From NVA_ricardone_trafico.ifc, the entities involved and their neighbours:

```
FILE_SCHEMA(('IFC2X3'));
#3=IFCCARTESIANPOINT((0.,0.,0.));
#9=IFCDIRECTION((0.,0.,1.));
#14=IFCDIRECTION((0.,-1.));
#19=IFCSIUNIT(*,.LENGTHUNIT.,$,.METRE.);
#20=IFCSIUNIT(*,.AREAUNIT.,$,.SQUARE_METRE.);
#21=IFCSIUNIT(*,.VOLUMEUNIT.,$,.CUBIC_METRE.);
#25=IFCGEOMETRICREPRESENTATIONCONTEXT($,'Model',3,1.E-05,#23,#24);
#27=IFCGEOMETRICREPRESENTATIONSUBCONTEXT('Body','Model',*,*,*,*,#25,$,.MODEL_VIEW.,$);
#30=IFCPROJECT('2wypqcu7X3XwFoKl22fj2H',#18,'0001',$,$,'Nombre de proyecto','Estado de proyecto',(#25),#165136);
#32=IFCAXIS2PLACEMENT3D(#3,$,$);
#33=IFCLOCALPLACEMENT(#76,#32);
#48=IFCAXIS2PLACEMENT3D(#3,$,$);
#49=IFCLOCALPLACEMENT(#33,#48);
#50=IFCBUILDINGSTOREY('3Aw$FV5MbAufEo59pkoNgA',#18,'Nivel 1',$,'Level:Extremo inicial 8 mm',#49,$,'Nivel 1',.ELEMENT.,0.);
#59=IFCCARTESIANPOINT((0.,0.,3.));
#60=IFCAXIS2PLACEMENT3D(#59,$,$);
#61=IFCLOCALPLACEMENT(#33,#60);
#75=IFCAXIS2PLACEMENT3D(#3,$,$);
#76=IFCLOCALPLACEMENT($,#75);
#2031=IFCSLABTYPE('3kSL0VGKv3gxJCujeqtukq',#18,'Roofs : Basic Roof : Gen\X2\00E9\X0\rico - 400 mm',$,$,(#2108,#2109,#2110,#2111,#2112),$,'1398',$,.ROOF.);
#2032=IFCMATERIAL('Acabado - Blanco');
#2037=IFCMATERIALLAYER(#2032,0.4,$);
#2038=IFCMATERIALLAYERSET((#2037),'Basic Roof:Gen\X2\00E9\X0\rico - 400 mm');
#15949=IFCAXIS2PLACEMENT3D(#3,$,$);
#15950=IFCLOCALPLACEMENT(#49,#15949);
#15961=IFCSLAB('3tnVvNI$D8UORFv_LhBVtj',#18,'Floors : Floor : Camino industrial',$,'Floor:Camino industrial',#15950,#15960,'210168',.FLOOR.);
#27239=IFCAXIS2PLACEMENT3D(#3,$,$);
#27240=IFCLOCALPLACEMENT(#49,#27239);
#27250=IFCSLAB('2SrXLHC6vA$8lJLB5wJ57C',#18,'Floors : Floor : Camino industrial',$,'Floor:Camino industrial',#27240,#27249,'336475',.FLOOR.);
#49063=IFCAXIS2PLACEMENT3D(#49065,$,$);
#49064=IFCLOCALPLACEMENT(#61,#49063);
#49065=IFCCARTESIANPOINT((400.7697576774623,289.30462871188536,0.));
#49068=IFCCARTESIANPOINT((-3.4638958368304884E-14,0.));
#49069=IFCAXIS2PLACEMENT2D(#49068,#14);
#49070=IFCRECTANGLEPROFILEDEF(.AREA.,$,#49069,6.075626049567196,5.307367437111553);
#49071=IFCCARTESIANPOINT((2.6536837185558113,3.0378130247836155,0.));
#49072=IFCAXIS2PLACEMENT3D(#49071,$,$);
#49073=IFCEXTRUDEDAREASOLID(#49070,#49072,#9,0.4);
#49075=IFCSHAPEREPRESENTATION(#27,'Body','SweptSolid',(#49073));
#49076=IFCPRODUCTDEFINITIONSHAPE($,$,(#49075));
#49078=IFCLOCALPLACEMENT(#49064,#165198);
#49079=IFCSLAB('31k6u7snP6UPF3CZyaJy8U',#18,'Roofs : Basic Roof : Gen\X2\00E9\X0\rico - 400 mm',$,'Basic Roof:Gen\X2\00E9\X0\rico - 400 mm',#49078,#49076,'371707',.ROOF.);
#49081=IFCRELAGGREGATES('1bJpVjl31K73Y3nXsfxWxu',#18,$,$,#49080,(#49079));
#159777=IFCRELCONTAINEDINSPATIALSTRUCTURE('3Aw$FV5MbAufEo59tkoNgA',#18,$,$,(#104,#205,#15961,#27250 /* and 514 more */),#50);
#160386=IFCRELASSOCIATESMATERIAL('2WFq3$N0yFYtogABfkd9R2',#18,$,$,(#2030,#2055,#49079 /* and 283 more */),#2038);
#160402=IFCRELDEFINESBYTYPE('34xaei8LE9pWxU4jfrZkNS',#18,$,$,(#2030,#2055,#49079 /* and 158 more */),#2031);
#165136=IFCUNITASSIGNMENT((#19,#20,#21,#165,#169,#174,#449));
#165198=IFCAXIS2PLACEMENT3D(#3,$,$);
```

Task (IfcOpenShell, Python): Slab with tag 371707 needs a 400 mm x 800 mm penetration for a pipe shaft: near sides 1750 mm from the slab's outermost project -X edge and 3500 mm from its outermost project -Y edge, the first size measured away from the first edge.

```python
import numpy as np
import ifcopenshell
import ifcopenshell.api.feature
import ifcopenshell.api.geometry
import ifcopenshell.api.root
import ifcopenshell.geom
import ifcopenshell.util.placement
import ifcopenshell.util.representation
import ifcopenshell.util.shape
import ifcopenshell.util.unit

model = ifcopenshell.open("NVA_ricardone_trafico.ifc")
unit_scale = ifcopenshell.util.unit.calculate_unit_scale(model)
settings = ifcopenshell.geom.settings()


def volume(element):
    """Net volume in cubic metres, openings subtracted."""
    shape = ifcopenshell.geom.create_shape(settings, element)
    return ifcopenshell.util.shape.get_volume(shape.geometry)


slab = model.by_id(49079)
before = volume(slab)

# Extent in the slab's own axes, in metres. The edges named are its -X and -Y sides.
slab_shape = ifcopenshell.geom.create_shape(settings, slab)
vertices = ifcopenshell.util.shape.get_vertices(slab_shape.geometry)
x_min, y_min, bottom = vertices.min(axis=0)
top = vertices[:, 2].max()

opening = ifcopenshell.api.root.create_entity(model, ifc_class="IfcOpeningElement", name="Pipe shaft opening")
context = ifcopenshell.util.representation.get_context(model, "Model", "Body", "MODEL_VIEW")
width, depth = 0.4, 0.8
outline = [(0.0, 0.0), (width, 0.0), (width, depth), (0.0, depth), (0.0, 0.0)]
# Overshoot both faces by 50 mm so the cut is clean.
shape = ifcopenshell.api.geometry.add_slab_representation(
    model, context=context, depth=top - bottom + 0.1, polyline=outline
)
ifcopenshell.api.geometry.assign_representation(model, product=opening, representation=shape)

matrix = ifcopenshell.util.placement.get_local_placement(slab.ObjectPlacement)
matrix[:, 3] = matrix @ np.append(np.array([x_min + 1.75, y_min + 3.5, bottom - 0.05]) / unit_scale, 1.0)
ifcopenshell.api.geometry.edit_object_placement(model, product=opening, matrix=matrix, is_si=False)
ifcopenshell.api.feature.add_feature(model, feature=opening, element=slab)

after = volume(slab)

print(f"slab volume {before:.3f} -> {after:.3f} m3")

model.write("NVA_ricardone_trafico_updated.ifc")
```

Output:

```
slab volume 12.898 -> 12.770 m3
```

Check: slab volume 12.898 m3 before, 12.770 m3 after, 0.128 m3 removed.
